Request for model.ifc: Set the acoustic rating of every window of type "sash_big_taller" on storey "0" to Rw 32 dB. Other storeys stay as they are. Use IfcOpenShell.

First a look at what the model holds.

```python
import ifcopenshell
import ifcopenshell.util.element

model = ifcopenshell.open("model.ifc")
print(model.schema)
storey = next(s for s in model.by_type("IfcBuildingStorey") if s.Name == "0")
windows = [e for e in ifcopenshell.util.element.get_decomposition(storey) if e.is_a("IfcWindow")]
seen = {}
for e in windows:
    element_type = ifcopenshell.util.element.get_type(e)
    key = (element_type.Name if element_type != e and element_type else None, ifcopenshell.util.element.get_pset(e, "Pset_WindowCommon", "AcousticRating"))
    seen[key] = seen.get(key, 0) + 1
for (name, value), count in sorted(seen.items(), key=str):
    print(count, "x", name, "|", value)
```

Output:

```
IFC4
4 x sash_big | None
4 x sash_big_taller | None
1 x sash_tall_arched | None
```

```python
import ifcopenshell
import ifcopenshell.api.pset
import ifcopenshell.util.element

model = ifcopenshell.open("model.ifc")

storey = next(s for s in model.by_type("IfcBuildingStorey") if s.Name == "0")
windows = [e for e in ifcopenshell.util.element.get_decomposition(storey) if e.is_a("IfcWindow")]

count = 0
for e in windows:
    element_type = ifcopenshell.util.element.get_type(e)
    if element_type in (None, e) or element_type.Name != "sash_big_taller":
        continue
    # add_pset returns the element's existing set when there is one.
    pset = ifcopenshell.api.pset.add_pset(model, product=e, name="Pset_WindowCommon")
    ifcopenshell.api.pset.edit_pset(model, pset=pset, properties={"AcousticRating": "Rw 32 dB"})
    count += 1

print(count, "windows updated")

model.write("model_v2.ifc")
```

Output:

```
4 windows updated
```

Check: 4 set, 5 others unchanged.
